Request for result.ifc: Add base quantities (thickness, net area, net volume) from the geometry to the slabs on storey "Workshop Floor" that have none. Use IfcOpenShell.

First a look at what the model holds.

```python
import ifcopenshell
import ifcopenshell.util.element
import ifcopenshell.util.unit

model = ifcopenshell.open("result.ifc")
print(model.schema)
for unit_type in ("LENGTHUNIT", "AREAUNIT", "VOLUMEUNIT"):
    print(unit_type, ifcopenshell.util.unit.calculate_unit_scale(model, unit_type))
storey = next(s for s in model.by_type("IfcBuildingStorey") if s.Name == "Workshop Floor")
slabs = [e for e in ifcopenshell.util.element.get_decomposition(storey) if e.is_a("IfcSlab")]
for e in sorted(slabs, key=lambda e: e.id()):
    print(e.id(), e.is_a(), e.Name, list(ifcopenshell.util.element.get_psets(e, qtos_only=True)), sep=" | ")
```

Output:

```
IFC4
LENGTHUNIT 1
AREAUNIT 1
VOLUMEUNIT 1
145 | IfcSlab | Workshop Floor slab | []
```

```python
import ifcopenshell
import ifcopenshell.api.pset
import ifcopenshell.geom
import ifcopenshell.util.element
import ifcopenshell.util.shape
import ifcopenshell.util.unit

model = ifcopenshell.open("result.ifc")
unit_scale = ifcopenshell.util.unit.calculate_unit_scale(model)
area_scale = ifcopenshell.util.unit.calculate_unit_scale(model, "AREAUNIT")
volume_scale = ifcopenshell.util.unit.calculate_unit_scale(model, "VOLUMEUNIT")
settings = ifcopenshell.geom.settings()

storey = next(s for s in model.by_type("IfcBuildingStorey") if s.Name == "Workshop Floor")
slabs = [e for e in ifcopenshell.util.element.get_decomposition(storey) if e.is_a("IfcSlab")]

for e in sorted(slabs, key=lambda e: e.id()):
    if ifcopenshell.util.element.get_psets(e, qtos_only=True, should_inherit=False):
        continue
    # Geometry comes back in metres, in the element's own axes.
    shape = ifcopenshell.geom.create_shape(settings, e)
    values = {
        "Width": ifcopenshell.util.shape.get_z(shape.geometry) / unit_scale,
        "NetArea": ifcopenshell.util.shape.get_footprint_area(shape.geometry) / area_scale,
        "NetVolume": ifcopenshell.util.shape.get_volume(shape.geometry) / volume_scale,
    }
    qto = ifcopenshell.api.pset.add_qto(model, product=e, name="Qto_SlabBaseQuantities")
    ifcopenshell.api.pset.edit_qto(model, qto=qto, properties=values)
    print(e.id(), {k: round(v, 3) for k, v in values.items()})

model.write("result-out.ifc")
```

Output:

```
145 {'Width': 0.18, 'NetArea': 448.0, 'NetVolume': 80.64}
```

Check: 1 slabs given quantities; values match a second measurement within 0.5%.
